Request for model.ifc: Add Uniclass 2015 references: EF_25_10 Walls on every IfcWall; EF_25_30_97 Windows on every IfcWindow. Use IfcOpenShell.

First a look at what the model holds.

```python
import ifcopenshell

model = ifcopenshell.open("model.ifc")
print(model.schema)
print("classifications:", [c.Name for c in model.by_type("IfcClassification")])
for ifc_class in ("IfcDoor", "IfcRoof", "IfcStair", "IfcWall", "IfcWindow"):
    print(ifc_class, len(model.by_type(ifc_class)))
```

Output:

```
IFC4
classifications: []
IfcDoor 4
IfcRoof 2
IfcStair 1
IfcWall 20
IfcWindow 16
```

```python
import ifcopenshell
import ifcopenshell.api.classification

model = ifcopenshell.open("model.ifc")

system = ifcopenshell.api.classification.add_classification(model, classification="Uniclass 2015")

codes = {
    "IfcWall": ("EF_25_10", "Walls"),
    "IfcWindow": ("EF_25_30_97", "Windows"),
}
for ifc_class, (code, name) in codes.items():
    products = model.by_type(ifc_class)
    ifcopenshell.api.classification.add_reference(
        model, products=products, classification=system, identification=code, name=name
    )
    print(code, len(products))

model.write("model_edited.ifc")
```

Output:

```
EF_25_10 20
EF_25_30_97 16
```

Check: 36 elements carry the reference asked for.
